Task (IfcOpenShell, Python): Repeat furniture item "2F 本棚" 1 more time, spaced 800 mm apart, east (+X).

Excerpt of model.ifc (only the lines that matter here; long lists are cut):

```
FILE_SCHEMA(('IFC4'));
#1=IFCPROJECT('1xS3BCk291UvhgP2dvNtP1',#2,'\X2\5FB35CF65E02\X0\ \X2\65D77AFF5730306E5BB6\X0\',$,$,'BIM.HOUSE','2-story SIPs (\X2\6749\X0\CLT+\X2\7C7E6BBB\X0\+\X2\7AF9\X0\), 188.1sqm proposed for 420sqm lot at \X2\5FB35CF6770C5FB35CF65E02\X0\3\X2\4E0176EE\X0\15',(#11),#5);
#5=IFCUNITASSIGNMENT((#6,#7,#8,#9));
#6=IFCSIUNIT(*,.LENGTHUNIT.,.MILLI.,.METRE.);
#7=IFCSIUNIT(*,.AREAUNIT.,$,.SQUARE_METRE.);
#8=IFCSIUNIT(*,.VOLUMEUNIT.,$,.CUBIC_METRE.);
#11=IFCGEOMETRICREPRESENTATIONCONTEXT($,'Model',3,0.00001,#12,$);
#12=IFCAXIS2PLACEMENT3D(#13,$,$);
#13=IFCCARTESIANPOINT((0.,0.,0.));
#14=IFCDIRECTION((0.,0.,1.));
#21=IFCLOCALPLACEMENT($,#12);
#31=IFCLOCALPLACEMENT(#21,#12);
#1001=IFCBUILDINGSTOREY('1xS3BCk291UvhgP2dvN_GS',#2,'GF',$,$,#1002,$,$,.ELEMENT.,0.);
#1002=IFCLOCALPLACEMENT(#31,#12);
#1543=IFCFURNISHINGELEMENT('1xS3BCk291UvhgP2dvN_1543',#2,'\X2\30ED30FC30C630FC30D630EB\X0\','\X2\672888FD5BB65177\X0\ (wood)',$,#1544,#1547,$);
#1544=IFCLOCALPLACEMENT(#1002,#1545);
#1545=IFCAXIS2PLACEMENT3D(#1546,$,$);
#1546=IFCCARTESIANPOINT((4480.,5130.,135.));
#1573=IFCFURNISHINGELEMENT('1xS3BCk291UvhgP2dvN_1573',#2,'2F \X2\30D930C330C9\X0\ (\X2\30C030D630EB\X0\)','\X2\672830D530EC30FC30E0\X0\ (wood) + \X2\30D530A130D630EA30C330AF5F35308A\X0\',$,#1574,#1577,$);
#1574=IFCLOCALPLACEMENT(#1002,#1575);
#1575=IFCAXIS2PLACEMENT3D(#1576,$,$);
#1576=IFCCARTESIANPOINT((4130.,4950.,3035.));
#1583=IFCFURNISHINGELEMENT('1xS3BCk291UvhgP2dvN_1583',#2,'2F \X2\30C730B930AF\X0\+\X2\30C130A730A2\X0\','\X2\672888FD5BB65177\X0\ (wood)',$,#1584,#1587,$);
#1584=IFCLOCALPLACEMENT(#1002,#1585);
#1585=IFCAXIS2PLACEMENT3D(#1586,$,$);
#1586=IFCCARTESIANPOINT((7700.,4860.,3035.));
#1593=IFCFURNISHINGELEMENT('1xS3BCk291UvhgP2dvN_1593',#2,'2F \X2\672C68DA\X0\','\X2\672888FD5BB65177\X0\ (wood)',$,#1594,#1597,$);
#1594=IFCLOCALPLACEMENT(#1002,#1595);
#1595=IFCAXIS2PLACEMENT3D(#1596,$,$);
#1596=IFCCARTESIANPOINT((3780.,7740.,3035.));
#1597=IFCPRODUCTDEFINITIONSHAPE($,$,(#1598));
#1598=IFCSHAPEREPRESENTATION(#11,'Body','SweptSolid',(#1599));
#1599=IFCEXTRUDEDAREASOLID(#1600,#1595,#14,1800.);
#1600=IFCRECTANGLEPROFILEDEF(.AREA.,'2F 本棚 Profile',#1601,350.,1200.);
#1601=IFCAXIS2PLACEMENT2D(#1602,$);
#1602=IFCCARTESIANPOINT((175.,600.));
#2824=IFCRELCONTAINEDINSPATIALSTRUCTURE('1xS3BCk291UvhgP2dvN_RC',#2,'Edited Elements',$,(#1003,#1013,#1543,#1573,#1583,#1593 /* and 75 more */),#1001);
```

```python
import numpy as np
import ifcopenshell
import ifcopenshell.api.geometry
import ifcopenshell.api.root
import ifcopenshell.util.element
import ifcopenshell.util.placement

model = ifcopenshell.open("model.ifc")


def reuse_history(source, copy):
    """copy_class also copies each property set's owner history, people and application; keep the originals."""
    for rel in copy.IsDefinedBy:
        if rel.is_a("IfcRelDefinesByProperties") and (history := rel.RelatingPropertyDefinition.OwnerHistory):
            rel.RelatingPropertyDefinition.OwnerHistory = source.OwnerHistory
            ifcopenshell.util.element.remove_deep2(model, history)


source = model.by_guid("1xS3BCk291UvhgP2dvN_1593")
base = ifcopenshell.util.placement.get_local_placement(source.ObjectPlacement)
step = np.array([1.0, 0.0, 0.0]) * 800.0

for i in range(1, 2):
    copy = ifcopenshell.api.root.copy_class(model, product=source)
    copy.Representation = ifcopenshell.util.element.copy_deep(
        model, source.Representation, exclude=["IfcGeometricRepresentationContext", "IfcRepresentationMap"]
    )
    reuse_history(source, copy)
    matrix = base.copy()
    matrix[:3, 3] += i * step
    print("added at", matrix[:3, 3].round(3) + 0.0)
    ifcopenshell.api.geometry.edit_object_placement(model, product=copy, matrix=matrix, is_si=False)

model.write("model-out.ifc")
```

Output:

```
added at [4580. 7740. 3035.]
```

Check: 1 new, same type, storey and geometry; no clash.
